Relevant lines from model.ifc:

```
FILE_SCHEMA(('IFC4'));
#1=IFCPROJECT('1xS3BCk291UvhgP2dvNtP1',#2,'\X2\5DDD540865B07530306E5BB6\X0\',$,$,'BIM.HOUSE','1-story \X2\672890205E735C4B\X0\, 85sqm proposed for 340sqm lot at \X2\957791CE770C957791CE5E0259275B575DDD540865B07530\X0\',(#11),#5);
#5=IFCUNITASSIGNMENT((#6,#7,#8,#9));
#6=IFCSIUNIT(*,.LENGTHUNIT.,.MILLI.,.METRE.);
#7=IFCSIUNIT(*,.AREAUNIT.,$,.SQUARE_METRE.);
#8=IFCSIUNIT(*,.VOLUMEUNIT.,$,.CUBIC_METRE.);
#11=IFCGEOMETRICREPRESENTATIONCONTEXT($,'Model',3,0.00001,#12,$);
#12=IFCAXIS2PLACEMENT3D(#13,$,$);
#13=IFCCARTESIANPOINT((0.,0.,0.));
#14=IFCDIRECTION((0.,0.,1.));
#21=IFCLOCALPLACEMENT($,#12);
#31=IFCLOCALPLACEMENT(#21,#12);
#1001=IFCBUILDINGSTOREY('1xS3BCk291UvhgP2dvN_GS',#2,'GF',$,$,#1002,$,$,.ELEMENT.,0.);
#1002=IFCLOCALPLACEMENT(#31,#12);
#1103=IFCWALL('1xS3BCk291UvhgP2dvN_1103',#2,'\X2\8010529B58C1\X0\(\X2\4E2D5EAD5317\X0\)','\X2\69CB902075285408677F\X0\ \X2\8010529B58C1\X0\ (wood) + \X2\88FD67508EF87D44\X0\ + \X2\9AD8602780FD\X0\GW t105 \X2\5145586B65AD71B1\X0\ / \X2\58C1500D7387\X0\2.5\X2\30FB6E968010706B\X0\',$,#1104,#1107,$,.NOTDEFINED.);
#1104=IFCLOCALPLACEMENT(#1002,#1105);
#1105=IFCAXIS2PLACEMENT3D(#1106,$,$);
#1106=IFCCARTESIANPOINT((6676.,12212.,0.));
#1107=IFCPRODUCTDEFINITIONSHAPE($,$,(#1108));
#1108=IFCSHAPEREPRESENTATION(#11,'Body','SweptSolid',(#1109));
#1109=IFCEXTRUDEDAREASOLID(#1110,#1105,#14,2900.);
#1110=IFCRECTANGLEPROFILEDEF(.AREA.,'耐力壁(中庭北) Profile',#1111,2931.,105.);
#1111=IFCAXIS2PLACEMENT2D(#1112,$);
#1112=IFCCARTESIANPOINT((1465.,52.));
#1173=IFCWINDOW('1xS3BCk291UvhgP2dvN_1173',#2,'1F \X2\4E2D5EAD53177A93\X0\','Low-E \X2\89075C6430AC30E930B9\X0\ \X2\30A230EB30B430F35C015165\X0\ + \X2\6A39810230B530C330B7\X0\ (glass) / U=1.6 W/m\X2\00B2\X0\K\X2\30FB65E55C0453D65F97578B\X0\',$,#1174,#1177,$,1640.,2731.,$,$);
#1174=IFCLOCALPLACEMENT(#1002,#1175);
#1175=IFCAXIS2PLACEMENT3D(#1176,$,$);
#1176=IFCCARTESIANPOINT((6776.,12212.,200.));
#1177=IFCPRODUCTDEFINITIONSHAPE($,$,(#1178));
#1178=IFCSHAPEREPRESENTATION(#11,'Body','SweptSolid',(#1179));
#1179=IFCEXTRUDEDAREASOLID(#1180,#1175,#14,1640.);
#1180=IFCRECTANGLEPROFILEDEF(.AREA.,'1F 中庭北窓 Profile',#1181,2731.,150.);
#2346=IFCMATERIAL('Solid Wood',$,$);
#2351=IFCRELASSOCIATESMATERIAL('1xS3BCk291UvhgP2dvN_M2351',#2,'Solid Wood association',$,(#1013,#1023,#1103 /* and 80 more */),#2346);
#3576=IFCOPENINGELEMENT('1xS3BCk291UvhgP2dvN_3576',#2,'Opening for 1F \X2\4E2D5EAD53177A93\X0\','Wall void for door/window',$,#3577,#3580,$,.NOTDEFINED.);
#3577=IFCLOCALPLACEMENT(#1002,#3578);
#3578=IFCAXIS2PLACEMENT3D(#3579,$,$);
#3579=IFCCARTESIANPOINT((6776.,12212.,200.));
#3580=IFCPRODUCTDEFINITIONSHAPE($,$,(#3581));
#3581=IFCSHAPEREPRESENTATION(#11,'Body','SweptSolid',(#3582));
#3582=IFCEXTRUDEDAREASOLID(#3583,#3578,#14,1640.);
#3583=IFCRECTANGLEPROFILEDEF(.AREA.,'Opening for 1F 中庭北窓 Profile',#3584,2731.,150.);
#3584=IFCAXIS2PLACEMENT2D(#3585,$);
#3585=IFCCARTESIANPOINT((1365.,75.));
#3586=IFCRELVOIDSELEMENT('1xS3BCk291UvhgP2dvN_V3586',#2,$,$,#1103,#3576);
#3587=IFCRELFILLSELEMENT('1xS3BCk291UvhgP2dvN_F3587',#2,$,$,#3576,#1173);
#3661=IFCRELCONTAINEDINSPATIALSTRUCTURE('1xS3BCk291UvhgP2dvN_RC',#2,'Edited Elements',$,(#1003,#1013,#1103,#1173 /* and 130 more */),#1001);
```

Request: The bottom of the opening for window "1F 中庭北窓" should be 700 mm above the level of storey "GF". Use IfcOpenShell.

```python
import numpy as np
import ifcopenshell
import ifcopenshell.api.geometry
import ifcopenshell.geom
import ifcopenshell.util.element
import ifcopenshell.util.placement
import ifcopenshell.util.shape
import ifcopenshell.util.unit

model = ifcopenshell.open("model.ifc")
unit_scale = ifcopenshell.util.unit.calculate_unit_scale(model)

window = model.by_id(1173)
opening = window.FillsVoids[0].RelatingOpeningElement
storey = ifcopenshell.util.element.get_container(window, ifc_class="IfcBuildingStorey")
level = ifcopenshell.util.placement.get_local_placement(storey.ObjectPlacement)[2, 3]

# The opening's origin need not be at the sill, so measure its lowest point.
shape = ifcopenshell.geom.create_shape(ifcopenshell.geom.settings(), opening)
bottom = ifcopenshell.util.shape.get_shape_bottom_elevation(shape, shape.geometry) / unit_scale
dz = level + 0.7 / unit_scale - bottom

shift = np.array([0.0, 0.0, dz])
# The window is not placed relative to its opening, so move both.
for product in (opening, window):
    matrix = ifcopenshell.util.placement.get_local_placement(product.ObjectPlacement)
    matrix[:3, 3] += shift
    ifcopenshell.api.geometry.edit_object_placement(model, product=product, matrix=matrix, is_si=False)

print(f"moved by {dz * unit_scale:+.3f} m")

model.write("model_updated.ifc")
```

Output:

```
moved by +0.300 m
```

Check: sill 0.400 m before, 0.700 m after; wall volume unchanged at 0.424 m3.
